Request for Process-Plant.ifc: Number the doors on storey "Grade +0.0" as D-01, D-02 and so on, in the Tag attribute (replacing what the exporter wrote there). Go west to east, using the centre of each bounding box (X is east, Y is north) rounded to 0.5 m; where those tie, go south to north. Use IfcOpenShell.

First a look at what the model holds.

```python
import ifcopenshell
import ifcopenshell.util.element
import ifcopenshell.util.placement

model = ifcopenshell.open("Process-Plant.ifc")
print(model.schema)
storey = next(s for s in model.by_type("IfcBuildingStorey") if s.Name == "Grade +0.0")
doors = [e for e in ifcopenshell.util.element.get_decomposition(storey) if e.is_a("IfcDoor")]
for e in sorted(doors, key=lambda e: e.id()):
    origin = ifcopenshell.util.placement.get_local_placement(e.ObjectPlacement)[:3, 3]
    print(e.id(), e.Tag, e.Name, origin.round(2) + 0.0, sep=" | ")
```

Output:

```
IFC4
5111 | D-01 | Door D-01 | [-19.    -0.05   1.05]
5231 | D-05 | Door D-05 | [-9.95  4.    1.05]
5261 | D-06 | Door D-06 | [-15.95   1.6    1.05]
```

```python
import ifcopenshell
import ifcopenshell.geom
import ifcopenshell.util.element
import ifcopenshell.util.shape

model = ifcopenshell.open("Process-Plant.ifc")
settings = ifcopenshell.geom.settings()
settings.set("use-world-coords", True)


def centre(element):
    shape = ifcopenshell.geom.create_shape(settings, element)
    return ifcopenshell.util.shape.get_bbox_centroid(shape.geometry)


storey = next(s for s in model.by_type("IfcBuildingStorey") if s.Name == "Grade +0.0")
doors = [e for e in ifcopenshell.util.element.get_decomposition(storey) if e.is_a("IfcDoor")]

# Insertion points can sit at a corner or the storey origin, so sort by the geometry (in metres).
centres = {e: centre(e) for e in doors}
doors.sort(key=lambda e: (round(centres[e][0] / 0.5), centres[e][1]))

for i, e in enumerate(doors, start=1):
    number = f"D-{i:02d}"
    e.Tag = number
    print(e.id(), number)

model.write("Process-Plant_updated.ifc")
```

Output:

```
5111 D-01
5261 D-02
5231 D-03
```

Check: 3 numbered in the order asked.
